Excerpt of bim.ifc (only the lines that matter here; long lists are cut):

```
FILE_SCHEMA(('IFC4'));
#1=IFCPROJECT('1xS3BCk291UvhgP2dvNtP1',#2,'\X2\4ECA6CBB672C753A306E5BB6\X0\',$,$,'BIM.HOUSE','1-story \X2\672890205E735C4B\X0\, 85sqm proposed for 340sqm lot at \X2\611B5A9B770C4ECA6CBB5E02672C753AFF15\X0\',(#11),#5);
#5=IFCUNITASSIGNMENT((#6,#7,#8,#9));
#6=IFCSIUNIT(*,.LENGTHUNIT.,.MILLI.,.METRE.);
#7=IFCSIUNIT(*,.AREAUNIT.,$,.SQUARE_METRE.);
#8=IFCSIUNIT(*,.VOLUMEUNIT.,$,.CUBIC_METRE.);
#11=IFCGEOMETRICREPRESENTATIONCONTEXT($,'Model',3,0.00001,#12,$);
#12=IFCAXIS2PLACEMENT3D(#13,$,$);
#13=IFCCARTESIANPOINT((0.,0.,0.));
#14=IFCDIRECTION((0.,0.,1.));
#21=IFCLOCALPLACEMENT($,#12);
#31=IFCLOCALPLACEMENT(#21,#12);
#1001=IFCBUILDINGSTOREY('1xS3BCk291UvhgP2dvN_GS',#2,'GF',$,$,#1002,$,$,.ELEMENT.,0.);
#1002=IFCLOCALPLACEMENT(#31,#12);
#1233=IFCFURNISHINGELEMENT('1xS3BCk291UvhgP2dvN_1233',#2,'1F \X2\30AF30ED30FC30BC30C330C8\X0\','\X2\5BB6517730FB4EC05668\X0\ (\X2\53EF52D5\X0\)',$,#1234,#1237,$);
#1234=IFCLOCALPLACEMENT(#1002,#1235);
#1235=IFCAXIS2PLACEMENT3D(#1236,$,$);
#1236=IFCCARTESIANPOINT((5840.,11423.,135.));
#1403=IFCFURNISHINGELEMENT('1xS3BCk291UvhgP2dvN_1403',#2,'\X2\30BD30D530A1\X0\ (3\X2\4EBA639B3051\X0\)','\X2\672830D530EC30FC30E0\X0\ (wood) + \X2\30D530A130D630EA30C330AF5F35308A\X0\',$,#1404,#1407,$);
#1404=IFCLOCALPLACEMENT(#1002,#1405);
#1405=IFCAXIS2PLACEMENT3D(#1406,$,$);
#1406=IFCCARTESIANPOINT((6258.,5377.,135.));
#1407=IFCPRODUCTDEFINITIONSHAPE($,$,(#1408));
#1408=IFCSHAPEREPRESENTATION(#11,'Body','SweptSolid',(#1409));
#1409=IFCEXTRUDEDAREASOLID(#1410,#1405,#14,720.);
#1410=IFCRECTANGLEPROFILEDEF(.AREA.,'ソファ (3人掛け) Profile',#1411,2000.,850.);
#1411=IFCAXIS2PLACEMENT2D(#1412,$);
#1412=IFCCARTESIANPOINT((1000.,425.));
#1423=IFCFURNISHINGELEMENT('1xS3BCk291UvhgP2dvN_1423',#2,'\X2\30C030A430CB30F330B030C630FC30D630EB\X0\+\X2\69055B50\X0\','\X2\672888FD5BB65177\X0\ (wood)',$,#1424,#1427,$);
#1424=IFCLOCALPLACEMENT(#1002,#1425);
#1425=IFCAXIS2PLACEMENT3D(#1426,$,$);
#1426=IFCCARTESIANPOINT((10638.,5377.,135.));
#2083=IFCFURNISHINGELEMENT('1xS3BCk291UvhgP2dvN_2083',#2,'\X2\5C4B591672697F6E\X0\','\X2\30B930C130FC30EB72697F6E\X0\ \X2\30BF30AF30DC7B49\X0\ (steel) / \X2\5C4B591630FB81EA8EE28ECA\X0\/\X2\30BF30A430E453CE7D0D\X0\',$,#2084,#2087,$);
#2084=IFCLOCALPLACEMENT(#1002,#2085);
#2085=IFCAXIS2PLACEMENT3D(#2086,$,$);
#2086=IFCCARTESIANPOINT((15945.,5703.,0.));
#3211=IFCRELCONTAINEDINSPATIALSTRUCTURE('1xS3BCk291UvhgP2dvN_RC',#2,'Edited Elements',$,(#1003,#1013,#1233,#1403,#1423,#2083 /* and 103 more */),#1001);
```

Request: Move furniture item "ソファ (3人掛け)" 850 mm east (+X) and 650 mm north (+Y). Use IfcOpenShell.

```python
import ifcopenshell
import ifcopenshell.api.geometry
import ifcopenshell.util.placement
import ifcopenshell.util.unit

model = ifcopenshell.open("bim.ifc")
unit_scale = ifcopenshell.util.unit.calculate_unit_scale(model)

item = model.by_guid("1xS3BCk291UvhgP2dvN_1403")
matrix = ifcopenshell.util.placement.get_local_placement(item.ObjectPlacement)
matrix[0, 3] += 0.85 / unit_scale
matrix[1, 3] += 0.65 / unit_scale
ifcopenshell.api.geometry.edit_object_placement(model, product=item, matrix=matrix, is_si=False)

print(ifcopenshell.util.placement.get_local_placement(item.ObjectPlacement).round(3) + 0.0)

model.write("bim-out.ifc")
```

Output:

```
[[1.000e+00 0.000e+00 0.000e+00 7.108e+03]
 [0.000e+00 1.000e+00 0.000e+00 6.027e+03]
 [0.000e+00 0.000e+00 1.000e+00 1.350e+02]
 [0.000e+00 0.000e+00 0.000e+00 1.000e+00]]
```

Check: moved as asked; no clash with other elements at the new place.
